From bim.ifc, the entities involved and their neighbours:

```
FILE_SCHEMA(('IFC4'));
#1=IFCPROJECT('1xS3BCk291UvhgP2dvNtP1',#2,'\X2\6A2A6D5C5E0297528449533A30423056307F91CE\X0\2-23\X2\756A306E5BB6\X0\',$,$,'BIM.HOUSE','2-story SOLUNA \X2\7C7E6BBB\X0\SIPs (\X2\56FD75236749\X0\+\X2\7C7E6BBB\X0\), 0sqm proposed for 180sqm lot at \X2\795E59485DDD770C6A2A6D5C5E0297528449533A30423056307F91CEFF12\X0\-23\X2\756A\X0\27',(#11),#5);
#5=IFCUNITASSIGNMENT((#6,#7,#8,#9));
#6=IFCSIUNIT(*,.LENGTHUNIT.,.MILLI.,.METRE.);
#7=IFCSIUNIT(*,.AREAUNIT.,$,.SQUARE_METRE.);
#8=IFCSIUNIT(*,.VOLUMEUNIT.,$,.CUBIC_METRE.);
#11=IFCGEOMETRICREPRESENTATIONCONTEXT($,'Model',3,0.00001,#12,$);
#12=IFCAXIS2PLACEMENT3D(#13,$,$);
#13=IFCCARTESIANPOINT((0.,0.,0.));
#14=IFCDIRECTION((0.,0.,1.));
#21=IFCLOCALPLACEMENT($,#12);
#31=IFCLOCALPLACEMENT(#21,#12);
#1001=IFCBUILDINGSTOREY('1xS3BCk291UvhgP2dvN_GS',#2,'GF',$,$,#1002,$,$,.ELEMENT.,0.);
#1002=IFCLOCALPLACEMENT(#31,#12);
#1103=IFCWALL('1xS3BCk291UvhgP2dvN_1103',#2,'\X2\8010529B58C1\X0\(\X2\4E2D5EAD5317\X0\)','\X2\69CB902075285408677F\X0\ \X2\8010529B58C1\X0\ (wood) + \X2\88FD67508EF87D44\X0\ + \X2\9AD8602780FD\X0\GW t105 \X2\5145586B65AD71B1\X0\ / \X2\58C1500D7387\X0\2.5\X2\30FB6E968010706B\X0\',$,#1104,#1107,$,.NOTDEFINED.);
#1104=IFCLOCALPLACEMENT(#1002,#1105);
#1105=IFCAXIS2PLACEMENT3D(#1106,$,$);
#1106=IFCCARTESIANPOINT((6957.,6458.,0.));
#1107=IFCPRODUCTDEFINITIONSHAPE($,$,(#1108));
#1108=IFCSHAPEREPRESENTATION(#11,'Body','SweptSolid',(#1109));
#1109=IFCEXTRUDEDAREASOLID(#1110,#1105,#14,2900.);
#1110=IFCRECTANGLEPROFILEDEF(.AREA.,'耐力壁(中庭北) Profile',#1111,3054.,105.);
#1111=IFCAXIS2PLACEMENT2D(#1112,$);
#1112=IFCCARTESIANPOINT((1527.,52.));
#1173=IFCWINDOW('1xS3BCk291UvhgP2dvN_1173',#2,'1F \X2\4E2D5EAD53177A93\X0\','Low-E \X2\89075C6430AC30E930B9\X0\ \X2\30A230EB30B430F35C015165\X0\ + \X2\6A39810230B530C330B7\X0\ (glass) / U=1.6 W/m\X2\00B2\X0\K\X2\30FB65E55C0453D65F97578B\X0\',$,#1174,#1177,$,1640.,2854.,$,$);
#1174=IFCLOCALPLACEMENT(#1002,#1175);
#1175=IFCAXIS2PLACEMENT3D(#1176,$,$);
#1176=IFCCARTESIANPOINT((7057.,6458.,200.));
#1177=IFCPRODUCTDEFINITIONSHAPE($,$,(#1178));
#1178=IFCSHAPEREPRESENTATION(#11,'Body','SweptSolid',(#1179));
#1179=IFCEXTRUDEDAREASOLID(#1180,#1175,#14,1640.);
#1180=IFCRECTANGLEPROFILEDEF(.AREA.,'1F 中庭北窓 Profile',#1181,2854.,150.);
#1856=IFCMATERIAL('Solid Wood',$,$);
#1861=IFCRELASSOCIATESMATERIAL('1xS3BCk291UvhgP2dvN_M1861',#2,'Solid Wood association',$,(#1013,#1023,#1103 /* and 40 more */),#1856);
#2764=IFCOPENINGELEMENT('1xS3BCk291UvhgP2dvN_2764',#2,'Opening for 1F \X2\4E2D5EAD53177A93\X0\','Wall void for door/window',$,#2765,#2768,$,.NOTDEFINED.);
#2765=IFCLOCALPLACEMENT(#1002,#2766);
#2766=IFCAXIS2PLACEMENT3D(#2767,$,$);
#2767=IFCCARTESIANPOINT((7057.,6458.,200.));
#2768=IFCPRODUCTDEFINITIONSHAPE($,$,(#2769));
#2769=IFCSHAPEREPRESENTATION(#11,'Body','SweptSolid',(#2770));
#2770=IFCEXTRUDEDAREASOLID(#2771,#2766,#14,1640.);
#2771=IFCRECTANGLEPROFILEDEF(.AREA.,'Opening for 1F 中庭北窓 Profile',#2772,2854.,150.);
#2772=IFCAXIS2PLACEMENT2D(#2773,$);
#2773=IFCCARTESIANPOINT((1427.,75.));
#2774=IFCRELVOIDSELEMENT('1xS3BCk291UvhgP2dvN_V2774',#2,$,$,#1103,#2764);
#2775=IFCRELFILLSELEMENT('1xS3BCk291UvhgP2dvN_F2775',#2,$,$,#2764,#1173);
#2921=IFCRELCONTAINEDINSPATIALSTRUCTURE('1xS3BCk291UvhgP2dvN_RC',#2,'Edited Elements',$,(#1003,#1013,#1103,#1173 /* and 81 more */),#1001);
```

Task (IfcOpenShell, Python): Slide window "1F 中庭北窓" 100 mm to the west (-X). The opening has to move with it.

```python
import ifcopenshell
import ifcopenshell.api.geometry
import ifcopenshell.util.placement
import ifcopenshell.util.unit

model = ifcopenshell.open("bim.ifc")
unit_scale = ifcopenshell.util.unit.calculate_unit_scale(model)

window = model.by_guid("1xS3BCk291UvhgP2dvN_1173")
opening = window.FillsVoids[0].RelatingOpeningElement
wall = opening.VoidsElements[0].RelatingBuildingElement

wall_matrix = ifcopenshell.util.placement.get_local_placement(wall.ObjectPlacement)
shift = wall_matrix[:3, 0] * -0.1 / unit_scale
before = ifcopenshell.util.placement.get_local_placement(window.ObjectPlacement)[:3, 3].copy()

# The window is not placed relative to its opening, so move both.
for product in (opening, window):
    matrix = ifcopenshell.util.placement.get_local_placement(product.ObjectPlacement)
    matrix[:3, 3] += shift
    ifcopenshell.api.geometry.edit_object_placement(model, product=product, matrix=matrix, is_si=False)

after = ifcopenshell.util.placement.get_local_placement(window.ObjectPlacement)[:3, 3]
print("window moved by", (after - before).round(3) + 0.0)

model.write("bim_v2.ifc")
```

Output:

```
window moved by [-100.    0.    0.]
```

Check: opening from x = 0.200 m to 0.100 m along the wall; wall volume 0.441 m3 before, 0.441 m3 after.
